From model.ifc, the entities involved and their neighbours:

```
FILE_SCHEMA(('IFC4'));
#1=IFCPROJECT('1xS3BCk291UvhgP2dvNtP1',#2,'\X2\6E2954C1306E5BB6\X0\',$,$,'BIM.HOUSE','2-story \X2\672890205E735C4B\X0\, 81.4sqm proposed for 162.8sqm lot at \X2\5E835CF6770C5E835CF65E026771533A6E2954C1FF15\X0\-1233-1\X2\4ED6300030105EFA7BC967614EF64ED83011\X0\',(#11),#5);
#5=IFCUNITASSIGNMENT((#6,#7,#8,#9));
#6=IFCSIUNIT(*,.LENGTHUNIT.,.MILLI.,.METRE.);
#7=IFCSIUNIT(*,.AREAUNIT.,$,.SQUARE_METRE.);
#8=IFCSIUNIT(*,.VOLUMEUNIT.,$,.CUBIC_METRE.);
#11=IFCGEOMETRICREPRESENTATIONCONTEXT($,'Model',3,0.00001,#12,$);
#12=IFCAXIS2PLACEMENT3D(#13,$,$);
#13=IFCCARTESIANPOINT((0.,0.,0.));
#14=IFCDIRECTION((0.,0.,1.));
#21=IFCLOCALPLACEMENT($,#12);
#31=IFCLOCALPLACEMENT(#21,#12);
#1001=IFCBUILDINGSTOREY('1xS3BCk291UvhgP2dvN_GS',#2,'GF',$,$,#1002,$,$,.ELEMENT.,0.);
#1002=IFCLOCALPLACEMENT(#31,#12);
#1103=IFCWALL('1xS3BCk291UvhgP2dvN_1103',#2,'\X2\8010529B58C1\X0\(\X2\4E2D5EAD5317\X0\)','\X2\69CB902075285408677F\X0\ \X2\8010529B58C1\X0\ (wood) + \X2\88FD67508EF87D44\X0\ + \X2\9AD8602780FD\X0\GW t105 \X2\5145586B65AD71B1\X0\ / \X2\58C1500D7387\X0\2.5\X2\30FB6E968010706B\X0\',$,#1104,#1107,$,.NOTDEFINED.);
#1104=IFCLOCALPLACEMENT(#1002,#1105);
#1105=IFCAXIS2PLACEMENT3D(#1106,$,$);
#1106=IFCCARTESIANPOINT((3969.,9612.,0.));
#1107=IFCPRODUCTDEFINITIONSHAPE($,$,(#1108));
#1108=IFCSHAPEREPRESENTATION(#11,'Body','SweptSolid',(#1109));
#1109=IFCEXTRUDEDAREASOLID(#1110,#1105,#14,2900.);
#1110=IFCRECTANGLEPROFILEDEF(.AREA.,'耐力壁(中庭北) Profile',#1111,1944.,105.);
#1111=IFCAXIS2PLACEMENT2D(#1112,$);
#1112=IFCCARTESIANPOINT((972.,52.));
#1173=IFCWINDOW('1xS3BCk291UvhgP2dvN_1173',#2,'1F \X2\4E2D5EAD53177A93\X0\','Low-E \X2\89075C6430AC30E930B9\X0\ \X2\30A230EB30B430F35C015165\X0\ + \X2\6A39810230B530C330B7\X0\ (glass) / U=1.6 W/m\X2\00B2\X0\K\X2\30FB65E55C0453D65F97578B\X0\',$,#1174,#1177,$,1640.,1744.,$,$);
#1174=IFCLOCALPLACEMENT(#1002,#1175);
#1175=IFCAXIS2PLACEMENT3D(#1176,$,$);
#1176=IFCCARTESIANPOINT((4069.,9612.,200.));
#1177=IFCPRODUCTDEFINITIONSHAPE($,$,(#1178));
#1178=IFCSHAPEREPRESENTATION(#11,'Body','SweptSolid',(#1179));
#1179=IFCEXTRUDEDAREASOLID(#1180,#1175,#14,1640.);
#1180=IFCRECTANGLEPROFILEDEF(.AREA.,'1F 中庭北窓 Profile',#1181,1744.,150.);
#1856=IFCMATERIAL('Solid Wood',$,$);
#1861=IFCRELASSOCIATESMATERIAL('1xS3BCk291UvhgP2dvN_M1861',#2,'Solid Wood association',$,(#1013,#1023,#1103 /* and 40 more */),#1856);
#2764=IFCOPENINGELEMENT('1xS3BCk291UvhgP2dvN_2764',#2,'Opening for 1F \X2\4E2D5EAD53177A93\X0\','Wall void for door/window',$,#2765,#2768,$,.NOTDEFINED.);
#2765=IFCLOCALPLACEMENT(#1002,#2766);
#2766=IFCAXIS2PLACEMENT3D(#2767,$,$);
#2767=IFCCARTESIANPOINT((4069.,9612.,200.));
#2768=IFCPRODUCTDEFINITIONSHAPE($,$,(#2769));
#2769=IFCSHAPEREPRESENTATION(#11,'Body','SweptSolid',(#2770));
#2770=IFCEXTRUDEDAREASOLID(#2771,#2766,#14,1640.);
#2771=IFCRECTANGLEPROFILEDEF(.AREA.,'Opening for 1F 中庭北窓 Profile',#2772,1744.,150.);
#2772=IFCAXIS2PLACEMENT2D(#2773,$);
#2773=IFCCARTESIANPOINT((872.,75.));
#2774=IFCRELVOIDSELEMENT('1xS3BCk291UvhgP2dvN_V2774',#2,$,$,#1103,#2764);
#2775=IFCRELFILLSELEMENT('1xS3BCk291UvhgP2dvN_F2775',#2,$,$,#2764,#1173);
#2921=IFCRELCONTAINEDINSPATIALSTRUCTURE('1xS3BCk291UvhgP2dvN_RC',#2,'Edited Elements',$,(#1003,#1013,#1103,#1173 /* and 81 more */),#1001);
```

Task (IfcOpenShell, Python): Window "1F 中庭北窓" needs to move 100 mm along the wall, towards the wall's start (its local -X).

```python
import ifcopenshell
import ifcopenshell.api.geometry
import ifcopenshell.util.placement
import ifcopenshell.util.unit

model = ifcopenshell.open("model.ifc")
unit_scale = ifcopenshell.util.unit.calculate_unit_scale(model)

window = model.by_guid("1xS3BCk291UvhgP2dvN_1173")
opening = window.FillsVoids[0].RelatingOpeningElement
wall = opening.VoidsElements[0].RelatingBuildingElement

wall_matrix = ifcopenshell.util.placement.get_local_placement(wall.ObjectPlacement)
shift = wall_matrix[:3, 0] * -0.1 / unit_scale
before = ifcopenshell.util.placement.get_local_placement(window.ObjectPlacement)[:3, 3].copy()

# The window is not placed relative to its opening, so move both.
for product in (opening, window):
    matrix = ifcopenshell.util.placement.get_local_placement(product.ObjectPlacement)
    matrix[:3, 3] += shift
    ifcopenshell.api.geometry.edit_object_placement(model, product=product, matrix=matrix, is_si=False)

after = ifcopenshell.util.placement.get_local_placement(window.ObjectPlacement)[:3, 3]
print("window moved by", (after - before).round(3) + 0.0)

model.write("model_edited.ifc")
```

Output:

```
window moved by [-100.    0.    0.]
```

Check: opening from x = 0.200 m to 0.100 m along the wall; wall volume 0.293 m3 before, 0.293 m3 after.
